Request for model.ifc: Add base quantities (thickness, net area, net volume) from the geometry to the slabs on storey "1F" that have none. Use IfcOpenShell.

First a look at what the model holds.

```python
import ifcopenshell
import ifcopenshell.util.element
import ifcopenshell.util.unit

model = ifcopenshell.open("model.ifc")
print(model.schema)
for unit_type in ("LENGTHUNIT", "AREAUNIT", "VOLUMEUNIT"):
    print(unit_type, ifcopenshell.util.unit.calculate_unit_scale(model, unit_type))
storey = next(s for s in model.by_type("IfcBuildingStorey") if s.Name == "1F")
slabs = [e for e in ifcopenshell.util.element.get_decomposition(storey) if e.is_a("IfcSlab")]
for e in sorted(slabs, key=lambda e: e.id()):
    print(e.id(), e.is_a(), e.Name, list(ifcopenshell.util.element.get_psets(e, qtos_only=True)), sep=" | ")
```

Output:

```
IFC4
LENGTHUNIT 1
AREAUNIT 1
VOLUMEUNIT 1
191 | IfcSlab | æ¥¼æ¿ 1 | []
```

```python
import ifcopenshell
import ifcopenshell.api.pset
import ifcopenshell.geom
import ifcopenshell.util.element
import ifcopenshell.util.shape
import ifcopenshell.util.unit

model = ifcopenshell.open("model.ifc")
unit_scale = ifcopenshell.util.unit.calculate_unit_scale(model)
area_scale = ifcopenshell.util.unit.calculate_unit_scale(model, "AREAUNIT")
volume_scale = ifcopenshell.util.unit.calculate_unit_scale(model, "VOLUMEUNIT")
settings = ifcopenshell.geom.settings()

storey = next(s for s in model.by_type("IfcBuildingStorey") if s.Name == "1F")
slabs = [e for e in ifcopenshell.util.element.get_decomposition(storey) if e.is_a("IfcSlab")]

for e in sorted(slabs, key=lambda e: e.id()):
    if ifcopenshell.util.element.get_psets(e, qtos_only=True, should_inherit=False):
        continue
    # Geometry comes back in metres, in the element's own axes.
    shape = ifcopenshell.geom.create_shape(settings, e)
    values = {
        "Width": ifcopenshell.util.shape.get_z(shape.geometry) / unit_scale,
        "NetArea": ifcopenshell.util.shape.get_footprint_area(shape.geometry) / area_scale,
        "NetVolume": ifcopenshell.util.shape.get_volume(shape.geometry) / volume_scale,
    }
    qto = ifcopenshell.api.pset.add_qto(model, product=e, name="Qto_SlabBaseQuantities")
    ifcopenshell.api.pset.edit_qto(model, qto=qto, properties=values)
    print(e.id(), {k: round(v, 3) for k, v in values.items()})

model.write("model_v2.ifc")
```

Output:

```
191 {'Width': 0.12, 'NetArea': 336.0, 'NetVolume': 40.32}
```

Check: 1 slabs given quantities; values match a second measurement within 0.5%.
